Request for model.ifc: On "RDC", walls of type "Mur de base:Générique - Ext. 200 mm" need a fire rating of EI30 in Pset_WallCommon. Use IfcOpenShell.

First a look at what the model holds.

```python
import ifcopenshell
import ifcopenshell.util.element

model = ifcopenshell.open("model.ifc")
print(model.schema)
storey = next(s for s in model.by_type("IfcBuildingStorey") if s.Name == "RDC")
walls = [e for e in ifcopenshell.util.element.get_decomposition(storey) if e.is_a("IfcWall")]
seen = {}
for e in walls:
    element_type = ifcopenshell.util.element.get_type(e)
    key = (element_type.Name if element_type != e and element_type else None, ifcopenshell.util.element.get_pset(e, "Pset_WallCommon", "FireRating"))
    seen[key] = seen.get(key, 0) + 1
for (name, value), count in sorted(seen.items(), key=str):
    print(count, "x", name, "|", value)
```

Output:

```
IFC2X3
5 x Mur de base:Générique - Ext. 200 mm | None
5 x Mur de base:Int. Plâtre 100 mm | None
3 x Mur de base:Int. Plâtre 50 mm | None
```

```python
import ifcopenshell
import ifcopenshell.api.pset
import ifcopenshell.util.element

model = ifcopenshell.open("model.ifc")

storey = next(s for s in model.by_type("IfcBuildingStorey") if s.Name == "RDC")
walls = [e for e in ifcopenshell.util.element.get_decomposition(storey) if e.is_a("IfcWall")]

count = 0
for e in walls:
    element_type = ifcopenshell.util.element.get_type(e)
    if element_type in (None, e) or element_type.Name != "Mur de base:Générique - Ext. 200 mm":
        continue
    # add_pset returns the element's existing set when there is one.
    pset = ifcopenshell.api.pset.add_pset(model, product=e, name="Pset_WallCommon")
    ifcopenshell.api.pset.edit_pset(model, pset=pset, properties={"FireRating": "EI30"})
    count += 1

print(count, "walls updated")

model.write("model_edited.ifc")
```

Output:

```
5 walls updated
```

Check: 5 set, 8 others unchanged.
